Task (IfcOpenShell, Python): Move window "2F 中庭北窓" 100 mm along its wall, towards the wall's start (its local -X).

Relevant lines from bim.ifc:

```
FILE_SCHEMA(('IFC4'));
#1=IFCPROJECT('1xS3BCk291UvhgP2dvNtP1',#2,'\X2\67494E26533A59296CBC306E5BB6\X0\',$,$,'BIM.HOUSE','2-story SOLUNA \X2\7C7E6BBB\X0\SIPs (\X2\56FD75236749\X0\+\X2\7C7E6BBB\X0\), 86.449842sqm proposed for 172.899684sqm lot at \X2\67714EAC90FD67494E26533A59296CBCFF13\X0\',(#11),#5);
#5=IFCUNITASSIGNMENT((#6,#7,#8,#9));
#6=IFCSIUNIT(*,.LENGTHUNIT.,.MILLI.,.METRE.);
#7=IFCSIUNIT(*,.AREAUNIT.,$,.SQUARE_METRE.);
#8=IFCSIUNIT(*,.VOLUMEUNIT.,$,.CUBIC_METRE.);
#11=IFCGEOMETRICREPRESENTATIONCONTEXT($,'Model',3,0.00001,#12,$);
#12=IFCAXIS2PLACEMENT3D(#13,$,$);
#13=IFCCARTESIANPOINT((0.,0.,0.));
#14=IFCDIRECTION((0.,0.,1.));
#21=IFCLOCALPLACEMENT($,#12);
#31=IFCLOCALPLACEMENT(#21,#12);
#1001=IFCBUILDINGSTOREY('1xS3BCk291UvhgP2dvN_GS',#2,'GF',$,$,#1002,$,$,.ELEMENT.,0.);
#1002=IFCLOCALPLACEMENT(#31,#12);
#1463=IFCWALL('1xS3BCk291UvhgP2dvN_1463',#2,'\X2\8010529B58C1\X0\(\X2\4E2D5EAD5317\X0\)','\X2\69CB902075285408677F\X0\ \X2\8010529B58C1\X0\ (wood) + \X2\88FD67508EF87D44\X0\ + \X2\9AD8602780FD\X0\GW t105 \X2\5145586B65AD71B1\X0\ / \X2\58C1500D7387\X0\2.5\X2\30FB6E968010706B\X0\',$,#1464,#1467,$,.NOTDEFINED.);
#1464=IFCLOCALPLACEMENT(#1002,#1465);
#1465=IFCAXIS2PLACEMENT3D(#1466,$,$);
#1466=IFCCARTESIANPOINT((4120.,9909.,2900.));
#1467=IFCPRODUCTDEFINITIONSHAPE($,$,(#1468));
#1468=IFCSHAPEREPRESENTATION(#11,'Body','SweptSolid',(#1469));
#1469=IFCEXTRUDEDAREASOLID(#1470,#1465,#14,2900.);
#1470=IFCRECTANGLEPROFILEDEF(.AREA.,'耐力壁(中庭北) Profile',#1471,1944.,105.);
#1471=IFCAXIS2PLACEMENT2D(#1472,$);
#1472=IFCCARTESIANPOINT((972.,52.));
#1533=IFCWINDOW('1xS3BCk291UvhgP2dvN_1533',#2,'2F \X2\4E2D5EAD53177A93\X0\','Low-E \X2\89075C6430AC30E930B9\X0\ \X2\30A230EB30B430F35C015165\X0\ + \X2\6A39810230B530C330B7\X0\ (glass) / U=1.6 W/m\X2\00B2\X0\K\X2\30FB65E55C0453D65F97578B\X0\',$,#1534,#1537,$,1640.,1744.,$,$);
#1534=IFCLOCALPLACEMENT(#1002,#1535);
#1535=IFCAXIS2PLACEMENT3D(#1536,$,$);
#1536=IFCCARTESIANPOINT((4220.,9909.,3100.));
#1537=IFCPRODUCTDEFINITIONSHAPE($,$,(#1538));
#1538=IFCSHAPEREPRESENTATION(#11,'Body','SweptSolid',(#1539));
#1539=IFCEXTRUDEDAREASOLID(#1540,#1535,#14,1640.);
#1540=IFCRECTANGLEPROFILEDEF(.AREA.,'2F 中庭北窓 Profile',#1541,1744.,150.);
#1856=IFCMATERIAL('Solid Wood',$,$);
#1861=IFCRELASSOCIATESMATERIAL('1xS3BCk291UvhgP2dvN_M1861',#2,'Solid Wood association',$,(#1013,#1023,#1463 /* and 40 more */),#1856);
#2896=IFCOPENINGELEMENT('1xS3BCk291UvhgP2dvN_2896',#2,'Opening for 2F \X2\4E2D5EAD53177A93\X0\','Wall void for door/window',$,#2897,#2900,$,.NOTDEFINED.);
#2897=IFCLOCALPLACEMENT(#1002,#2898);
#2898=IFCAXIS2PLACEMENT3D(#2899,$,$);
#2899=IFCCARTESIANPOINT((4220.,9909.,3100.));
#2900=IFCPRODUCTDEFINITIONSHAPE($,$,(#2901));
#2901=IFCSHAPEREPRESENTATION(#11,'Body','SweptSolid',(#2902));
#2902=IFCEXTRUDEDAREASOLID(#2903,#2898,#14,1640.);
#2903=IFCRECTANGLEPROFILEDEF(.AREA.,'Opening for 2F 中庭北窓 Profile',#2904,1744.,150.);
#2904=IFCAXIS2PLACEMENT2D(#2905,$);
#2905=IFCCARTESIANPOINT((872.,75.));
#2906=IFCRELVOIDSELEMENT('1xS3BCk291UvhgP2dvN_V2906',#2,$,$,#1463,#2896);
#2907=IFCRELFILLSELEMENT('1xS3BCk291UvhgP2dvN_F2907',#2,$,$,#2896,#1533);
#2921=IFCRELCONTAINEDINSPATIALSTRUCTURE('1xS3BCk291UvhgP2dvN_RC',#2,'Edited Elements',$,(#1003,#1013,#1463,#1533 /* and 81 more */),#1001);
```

```python
import ifcopenshell
import ifcopenshell.api.geometry
import ifcopenshell.util.placement
import ifcopenshell.util.unit

model = ifcopenshell.open("bim.ifc")
unit_scale = ifcopenshell.util.unit.calculate_unit_scale(model)

window = model.by_guid("1xS3BCk291UvhgP2dvN_1533")
opening = window.FillsVoids[0].RelatingOpeningElement
wall = opening.VoidsElements[0].RelatingBuildingElement

wall_matrix = ifcopenshell.util.placement.get_local_placement(wall.ObjectPlacement)
shift = wall_matrix[:3, 0] * -0.1 / unit_scale
before = ifcopenshell.util.placement.get_local_placement(window.ObjectPlacement)[:3, 3].copy()

# The window is not placed relative to its opening, so move both.
for product in (opening, window):
    matrix = ifcopenshell.util.placement.get_local_placement(product.ObjectPlacement)
    matrix[:3, 3] += shift
    ifcopenshell.api.geometry.edit_object_placement(model, product=product, matrix=matrix, is_si=False)

after = ifcopenshell.util.placement.get_local_placement(window.ObjectPlacement)[:3, 3]
print("window moved by", (after - before).round(3) + 0.0)

model.write("bim-out.ifc")
```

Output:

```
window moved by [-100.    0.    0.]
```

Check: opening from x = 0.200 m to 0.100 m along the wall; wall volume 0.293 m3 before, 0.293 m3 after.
